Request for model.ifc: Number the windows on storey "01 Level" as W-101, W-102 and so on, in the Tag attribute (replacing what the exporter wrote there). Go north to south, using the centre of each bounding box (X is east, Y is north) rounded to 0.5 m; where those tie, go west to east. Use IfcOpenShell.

First a look at what the model holds.

```python
import ifcopenshell
import ifcopenshell.util.element
import ifcopenshell.util.placement

model = ifcopenshell.open("model.ifc")
print(model.schema)
storey = next(s for s in model.by_type("IfcBuildingStorey") if s.Name == "01 Level")
windows = [e for e in ifcopenshell.util.element.get_decomposition(storey) if e.is_a("IfcWindow")]
for e in sorted(windows, key=lambda e: e.id()):
    origin = ifcopenshell.util.placement.get_local_placement(e.ObjectPlacement)[:3, 3]
    print(e.id(), e.Tag, e.Name, origin.round(2) + 0.0, sep=" | ")
```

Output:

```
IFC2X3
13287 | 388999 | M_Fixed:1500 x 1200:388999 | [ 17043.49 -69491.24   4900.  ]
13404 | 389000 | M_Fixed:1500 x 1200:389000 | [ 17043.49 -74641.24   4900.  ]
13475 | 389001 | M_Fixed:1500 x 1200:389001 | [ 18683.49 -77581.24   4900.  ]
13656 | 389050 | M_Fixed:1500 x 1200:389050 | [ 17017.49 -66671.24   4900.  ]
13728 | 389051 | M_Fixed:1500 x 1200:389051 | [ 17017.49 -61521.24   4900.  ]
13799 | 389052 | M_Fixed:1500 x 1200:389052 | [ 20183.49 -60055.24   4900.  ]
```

```python
import ifcopenshell
import ifcopenshell.geom
import ifcopenshell.util.element
import ifcopenshell.util.shape

model = ifcopenshell.open("model.ifc")
settings = ifcopenshell.geom.settings()
settings.set("use-world-coords", True)


def centre(element):
    shape = ifcopenshell.geom.create_shape(settings, element)
    return ifcopenshell.util.shape.get_bbox_centroid(shape.geometry)


storey = next(s for s in model.by_type("IfcBuildingStorey") if s.Name == "01 Level")
windows = [e for e in ifcopenshell.util.element.get_decomposition(storey) if e.is_a("IfcWindow")]

# Insertion points can sit at a corner or the storey origin, so sort by the geometry (in metres).
centres = {e: centre(e) for e in windows}
windows.sort(key=lambda e: (-round(centres[e][1] / 0.5), centres[e][0]))

for i, e in enumerate(windows, start=1):
    number = f"W-1{i:02d}"
    e.Tag = number
    print(e.id(), number)

model.write("model-out.ifc")
```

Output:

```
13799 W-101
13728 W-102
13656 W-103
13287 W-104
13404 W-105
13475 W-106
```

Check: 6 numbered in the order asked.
